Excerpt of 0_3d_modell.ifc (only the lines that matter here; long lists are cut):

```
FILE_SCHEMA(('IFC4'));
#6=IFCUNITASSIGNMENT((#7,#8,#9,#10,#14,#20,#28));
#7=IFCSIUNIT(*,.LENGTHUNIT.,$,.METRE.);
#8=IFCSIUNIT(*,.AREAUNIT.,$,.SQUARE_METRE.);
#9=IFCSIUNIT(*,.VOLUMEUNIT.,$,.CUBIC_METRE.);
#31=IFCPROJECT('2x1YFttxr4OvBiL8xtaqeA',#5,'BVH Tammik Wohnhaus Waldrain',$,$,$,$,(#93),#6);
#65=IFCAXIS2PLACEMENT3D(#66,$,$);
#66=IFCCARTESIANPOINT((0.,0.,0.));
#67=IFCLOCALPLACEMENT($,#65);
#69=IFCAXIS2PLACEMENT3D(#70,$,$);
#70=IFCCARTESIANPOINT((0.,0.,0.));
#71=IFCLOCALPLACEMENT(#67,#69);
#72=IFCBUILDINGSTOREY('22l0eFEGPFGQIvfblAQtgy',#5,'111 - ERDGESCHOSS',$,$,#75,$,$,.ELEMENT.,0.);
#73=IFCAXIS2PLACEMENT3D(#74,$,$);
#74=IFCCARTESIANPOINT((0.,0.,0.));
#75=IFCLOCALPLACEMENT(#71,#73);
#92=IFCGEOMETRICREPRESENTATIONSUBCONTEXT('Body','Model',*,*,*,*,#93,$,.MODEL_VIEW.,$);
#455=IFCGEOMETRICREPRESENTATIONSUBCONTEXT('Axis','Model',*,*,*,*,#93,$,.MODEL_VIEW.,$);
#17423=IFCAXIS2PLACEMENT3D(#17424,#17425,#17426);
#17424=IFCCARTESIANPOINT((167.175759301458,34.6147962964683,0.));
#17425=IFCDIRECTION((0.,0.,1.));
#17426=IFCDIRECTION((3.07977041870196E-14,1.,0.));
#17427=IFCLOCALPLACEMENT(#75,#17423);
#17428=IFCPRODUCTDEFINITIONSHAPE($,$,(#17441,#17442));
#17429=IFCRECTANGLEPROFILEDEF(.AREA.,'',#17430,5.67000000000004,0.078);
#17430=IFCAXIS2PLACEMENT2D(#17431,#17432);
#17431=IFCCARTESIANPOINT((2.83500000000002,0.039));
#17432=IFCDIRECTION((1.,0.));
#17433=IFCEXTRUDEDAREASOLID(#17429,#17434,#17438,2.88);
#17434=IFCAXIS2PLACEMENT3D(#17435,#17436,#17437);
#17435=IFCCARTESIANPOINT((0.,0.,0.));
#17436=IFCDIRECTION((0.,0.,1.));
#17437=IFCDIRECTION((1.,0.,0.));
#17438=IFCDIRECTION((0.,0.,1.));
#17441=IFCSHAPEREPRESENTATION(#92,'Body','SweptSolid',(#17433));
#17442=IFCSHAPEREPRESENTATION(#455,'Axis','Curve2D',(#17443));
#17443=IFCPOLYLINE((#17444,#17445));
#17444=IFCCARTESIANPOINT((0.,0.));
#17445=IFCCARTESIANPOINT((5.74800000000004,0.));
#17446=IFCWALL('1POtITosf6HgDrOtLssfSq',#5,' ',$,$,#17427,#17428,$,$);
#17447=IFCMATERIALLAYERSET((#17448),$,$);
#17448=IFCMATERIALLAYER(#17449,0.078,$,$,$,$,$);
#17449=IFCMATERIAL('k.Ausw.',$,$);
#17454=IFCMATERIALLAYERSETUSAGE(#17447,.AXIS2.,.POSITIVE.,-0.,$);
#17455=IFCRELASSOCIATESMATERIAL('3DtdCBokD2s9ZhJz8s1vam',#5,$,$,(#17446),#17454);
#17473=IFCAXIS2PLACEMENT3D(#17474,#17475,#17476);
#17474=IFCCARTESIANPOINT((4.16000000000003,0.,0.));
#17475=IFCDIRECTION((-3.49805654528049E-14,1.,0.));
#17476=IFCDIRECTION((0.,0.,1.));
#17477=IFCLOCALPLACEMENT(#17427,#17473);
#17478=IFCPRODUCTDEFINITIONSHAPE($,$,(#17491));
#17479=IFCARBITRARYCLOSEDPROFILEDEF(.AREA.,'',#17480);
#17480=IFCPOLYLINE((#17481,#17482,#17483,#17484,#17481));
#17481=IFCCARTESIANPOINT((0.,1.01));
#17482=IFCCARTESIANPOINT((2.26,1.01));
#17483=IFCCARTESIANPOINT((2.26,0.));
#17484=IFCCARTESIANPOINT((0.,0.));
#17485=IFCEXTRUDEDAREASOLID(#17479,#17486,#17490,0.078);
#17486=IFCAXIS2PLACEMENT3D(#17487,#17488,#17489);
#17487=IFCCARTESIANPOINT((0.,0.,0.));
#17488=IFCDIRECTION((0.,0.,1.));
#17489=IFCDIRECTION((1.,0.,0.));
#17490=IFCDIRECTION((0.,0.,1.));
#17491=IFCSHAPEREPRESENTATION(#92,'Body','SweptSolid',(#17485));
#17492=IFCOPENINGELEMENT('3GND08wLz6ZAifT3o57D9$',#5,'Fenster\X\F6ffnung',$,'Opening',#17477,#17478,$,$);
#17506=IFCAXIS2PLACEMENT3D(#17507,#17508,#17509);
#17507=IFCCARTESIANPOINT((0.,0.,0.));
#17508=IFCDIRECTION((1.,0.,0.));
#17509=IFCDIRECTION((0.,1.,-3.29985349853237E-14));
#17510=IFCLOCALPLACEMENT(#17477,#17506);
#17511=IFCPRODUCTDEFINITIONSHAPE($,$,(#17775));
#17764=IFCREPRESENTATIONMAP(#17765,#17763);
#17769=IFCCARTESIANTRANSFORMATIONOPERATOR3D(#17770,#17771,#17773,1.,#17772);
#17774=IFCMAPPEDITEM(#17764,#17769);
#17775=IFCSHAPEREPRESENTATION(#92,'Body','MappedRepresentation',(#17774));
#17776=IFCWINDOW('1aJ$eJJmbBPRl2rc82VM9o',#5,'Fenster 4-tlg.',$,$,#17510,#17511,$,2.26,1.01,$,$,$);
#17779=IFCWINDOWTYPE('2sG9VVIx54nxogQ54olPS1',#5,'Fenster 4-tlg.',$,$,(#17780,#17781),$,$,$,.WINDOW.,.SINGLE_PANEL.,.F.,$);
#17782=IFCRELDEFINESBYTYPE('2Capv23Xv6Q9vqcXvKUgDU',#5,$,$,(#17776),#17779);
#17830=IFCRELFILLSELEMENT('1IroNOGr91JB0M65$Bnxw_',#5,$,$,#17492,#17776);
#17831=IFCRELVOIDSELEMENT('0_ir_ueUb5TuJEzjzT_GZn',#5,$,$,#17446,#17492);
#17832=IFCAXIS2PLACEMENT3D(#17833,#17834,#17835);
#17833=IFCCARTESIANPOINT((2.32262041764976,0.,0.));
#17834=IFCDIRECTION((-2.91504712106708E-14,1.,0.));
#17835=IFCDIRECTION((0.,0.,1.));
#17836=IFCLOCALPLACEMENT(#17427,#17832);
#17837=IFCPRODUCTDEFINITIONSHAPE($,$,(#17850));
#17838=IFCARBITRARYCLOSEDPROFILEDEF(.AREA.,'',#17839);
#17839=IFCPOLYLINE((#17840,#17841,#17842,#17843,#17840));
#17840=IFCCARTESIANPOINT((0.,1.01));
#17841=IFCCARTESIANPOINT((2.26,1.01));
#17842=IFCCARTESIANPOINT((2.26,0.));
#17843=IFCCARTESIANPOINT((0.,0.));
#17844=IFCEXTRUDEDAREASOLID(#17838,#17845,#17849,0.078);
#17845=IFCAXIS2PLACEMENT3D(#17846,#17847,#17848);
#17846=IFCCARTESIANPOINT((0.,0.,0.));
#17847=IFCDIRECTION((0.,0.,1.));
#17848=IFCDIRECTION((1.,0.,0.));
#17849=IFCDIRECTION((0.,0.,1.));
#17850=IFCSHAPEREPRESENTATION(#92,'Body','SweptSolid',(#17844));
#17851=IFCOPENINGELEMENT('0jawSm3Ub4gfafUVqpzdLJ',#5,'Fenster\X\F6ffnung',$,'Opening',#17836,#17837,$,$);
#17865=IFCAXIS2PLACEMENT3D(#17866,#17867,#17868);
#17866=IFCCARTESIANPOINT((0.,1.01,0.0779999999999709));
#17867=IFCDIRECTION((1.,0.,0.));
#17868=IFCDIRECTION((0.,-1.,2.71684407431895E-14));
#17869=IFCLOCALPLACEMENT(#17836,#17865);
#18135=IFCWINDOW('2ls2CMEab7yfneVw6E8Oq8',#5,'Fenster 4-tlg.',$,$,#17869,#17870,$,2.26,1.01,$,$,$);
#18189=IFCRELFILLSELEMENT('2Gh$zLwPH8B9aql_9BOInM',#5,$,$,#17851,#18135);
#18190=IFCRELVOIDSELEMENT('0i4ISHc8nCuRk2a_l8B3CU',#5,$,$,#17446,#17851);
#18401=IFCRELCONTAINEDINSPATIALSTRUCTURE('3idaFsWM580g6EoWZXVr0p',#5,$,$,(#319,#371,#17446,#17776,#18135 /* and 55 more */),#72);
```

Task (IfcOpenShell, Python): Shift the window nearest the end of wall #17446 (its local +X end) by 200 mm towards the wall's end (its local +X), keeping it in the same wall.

```python
import ifcopenshell
import ifcopenshell.api.geometry
import ifcopenshell.util.placement

model = ifcopenshell.open("0_3d_modell.ifc")

window = model.by_id(17776)
opening = window.FillsVoids[0].RelatingOpeningElement
wall = opening.VoidsElements[0].RelatingBuildingElement

wall_matrix = ifcopenshell.util.placement.get_local_placement(wall.ObjectPlacement)
shift = wall_matrix[:3, 0] * 0.2
before = ifcopenshell.util.placement.get_local_placement(window.ObjectPlacement)[:3, 3].copy()

# The window is placed relative to its opening, so it follows when the opening moves.
matrix = ifcopenshell.util.placement.get_local_placement(opening.ObjectPlacement)
matrix[:3, 3] += shift
ifcopenshell.api.geometry.edit_object_placement(
    model, product=opening, matrix=matrix, is_si=False, should_transform_children=True
)

after = ifcopenshell.util.placement.get_local_placement(window.ObjectPlacement)[:3, 3]
print("window moved by", (after - before).round(3) + 0.0)

model.write("0_3d_modell-out.ifc")
```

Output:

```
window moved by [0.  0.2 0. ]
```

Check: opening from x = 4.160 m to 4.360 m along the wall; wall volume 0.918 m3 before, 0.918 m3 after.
